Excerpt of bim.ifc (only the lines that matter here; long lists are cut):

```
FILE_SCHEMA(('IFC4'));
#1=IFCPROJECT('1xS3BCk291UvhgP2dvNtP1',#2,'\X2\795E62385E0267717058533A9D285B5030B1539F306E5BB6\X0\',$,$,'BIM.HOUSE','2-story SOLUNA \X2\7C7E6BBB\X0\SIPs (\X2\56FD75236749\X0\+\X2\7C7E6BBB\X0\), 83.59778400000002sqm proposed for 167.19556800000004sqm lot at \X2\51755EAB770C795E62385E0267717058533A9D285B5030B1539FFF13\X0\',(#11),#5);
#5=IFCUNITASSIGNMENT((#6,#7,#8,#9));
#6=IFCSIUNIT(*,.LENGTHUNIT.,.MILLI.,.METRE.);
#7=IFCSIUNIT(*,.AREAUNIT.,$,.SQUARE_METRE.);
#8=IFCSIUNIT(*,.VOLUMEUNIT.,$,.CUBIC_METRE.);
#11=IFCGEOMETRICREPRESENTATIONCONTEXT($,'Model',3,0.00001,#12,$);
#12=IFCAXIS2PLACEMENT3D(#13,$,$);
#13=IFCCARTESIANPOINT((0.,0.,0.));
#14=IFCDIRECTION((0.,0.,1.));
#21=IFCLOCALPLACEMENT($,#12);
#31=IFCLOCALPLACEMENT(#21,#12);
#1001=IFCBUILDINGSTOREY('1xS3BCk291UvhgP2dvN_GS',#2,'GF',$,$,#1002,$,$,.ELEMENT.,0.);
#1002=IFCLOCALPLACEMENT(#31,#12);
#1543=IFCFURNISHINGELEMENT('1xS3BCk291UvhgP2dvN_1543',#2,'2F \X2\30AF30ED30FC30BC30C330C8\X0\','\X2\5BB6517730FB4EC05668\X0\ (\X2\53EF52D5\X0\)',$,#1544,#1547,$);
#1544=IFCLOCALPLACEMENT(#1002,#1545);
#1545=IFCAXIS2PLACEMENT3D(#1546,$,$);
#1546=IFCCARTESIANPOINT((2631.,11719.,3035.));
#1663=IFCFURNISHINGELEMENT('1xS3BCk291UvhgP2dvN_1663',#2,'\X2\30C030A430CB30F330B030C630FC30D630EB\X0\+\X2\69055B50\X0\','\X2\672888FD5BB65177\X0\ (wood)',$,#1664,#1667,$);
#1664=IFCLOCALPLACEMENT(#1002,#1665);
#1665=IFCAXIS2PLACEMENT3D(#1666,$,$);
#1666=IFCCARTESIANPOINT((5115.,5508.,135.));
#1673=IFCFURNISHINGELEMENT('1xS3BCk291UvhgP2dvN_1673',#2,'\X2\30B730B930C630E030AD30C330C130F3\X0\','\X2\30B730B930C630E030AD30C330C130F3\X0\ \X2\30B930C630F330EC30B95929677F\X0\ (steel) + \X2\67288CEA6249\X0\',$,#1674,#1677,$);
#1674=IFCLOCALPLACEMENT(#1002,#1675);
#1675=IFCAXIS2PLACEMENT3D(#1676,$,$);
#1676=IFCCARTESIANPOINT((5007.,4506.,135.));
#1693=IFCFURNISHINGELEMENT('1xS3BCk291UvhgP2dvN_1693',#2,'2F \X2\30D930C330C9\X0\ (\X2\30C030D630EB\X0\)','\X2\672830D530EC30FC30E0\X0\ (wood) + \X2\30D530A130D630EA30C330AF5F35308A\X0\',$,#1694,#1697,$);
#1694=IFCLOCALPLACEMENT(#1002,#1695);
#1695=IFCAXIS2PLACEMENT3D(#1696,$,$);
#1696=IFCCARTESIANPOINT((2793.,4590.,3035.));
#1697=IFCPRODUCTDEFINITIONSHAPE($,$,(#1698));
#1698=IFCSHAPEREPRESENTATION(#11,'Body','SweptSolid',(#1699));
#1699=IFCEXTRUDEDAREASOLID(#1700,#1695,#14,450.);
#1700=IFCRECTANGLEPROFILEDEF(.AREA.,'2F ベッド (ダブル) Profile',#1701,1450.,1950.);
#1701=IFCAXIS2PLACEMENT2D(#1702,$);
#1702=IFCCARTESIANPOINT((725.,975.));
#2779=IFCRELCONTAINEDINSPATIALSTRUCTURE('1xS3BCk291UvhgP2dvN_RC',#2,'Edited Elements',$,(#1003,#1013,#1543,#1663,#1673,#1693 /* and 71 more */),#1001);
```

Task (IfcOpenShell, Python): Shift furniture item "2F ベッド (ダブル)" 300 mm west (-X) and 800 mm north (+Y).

```python
import ifcopenshell
import ifcopenshell.api.geometry
import ifcopenshell.util.placement

model = ifcopenshell.open("bim.ifc")

item = model.by_guid("1xS3BCk291UvhgP2dvN_1693")
matrix = ifcopenshell.util.placement.get_local_placement(item.ObjectPlacement)
matrix[0, 3] -= 300.0
matrix[1, 3] += 800.0
ifcopenshell.api.geometry.edit_object_placement(model, product=item, matrix=matrix, is_si=False)

print(ifcopenshell.util.placement.get_local_placement(item.ObjectPlacement).round(3) + 0.0)

model.write("bim_updated.ifc")
```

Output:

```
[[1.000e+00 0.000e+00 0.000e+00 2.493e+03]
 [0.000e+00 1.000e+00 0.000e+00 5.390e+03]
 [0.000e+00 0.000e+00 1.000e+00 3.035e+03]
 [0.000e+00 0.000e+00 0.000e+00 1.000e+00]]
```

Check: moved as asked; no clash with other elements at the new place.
